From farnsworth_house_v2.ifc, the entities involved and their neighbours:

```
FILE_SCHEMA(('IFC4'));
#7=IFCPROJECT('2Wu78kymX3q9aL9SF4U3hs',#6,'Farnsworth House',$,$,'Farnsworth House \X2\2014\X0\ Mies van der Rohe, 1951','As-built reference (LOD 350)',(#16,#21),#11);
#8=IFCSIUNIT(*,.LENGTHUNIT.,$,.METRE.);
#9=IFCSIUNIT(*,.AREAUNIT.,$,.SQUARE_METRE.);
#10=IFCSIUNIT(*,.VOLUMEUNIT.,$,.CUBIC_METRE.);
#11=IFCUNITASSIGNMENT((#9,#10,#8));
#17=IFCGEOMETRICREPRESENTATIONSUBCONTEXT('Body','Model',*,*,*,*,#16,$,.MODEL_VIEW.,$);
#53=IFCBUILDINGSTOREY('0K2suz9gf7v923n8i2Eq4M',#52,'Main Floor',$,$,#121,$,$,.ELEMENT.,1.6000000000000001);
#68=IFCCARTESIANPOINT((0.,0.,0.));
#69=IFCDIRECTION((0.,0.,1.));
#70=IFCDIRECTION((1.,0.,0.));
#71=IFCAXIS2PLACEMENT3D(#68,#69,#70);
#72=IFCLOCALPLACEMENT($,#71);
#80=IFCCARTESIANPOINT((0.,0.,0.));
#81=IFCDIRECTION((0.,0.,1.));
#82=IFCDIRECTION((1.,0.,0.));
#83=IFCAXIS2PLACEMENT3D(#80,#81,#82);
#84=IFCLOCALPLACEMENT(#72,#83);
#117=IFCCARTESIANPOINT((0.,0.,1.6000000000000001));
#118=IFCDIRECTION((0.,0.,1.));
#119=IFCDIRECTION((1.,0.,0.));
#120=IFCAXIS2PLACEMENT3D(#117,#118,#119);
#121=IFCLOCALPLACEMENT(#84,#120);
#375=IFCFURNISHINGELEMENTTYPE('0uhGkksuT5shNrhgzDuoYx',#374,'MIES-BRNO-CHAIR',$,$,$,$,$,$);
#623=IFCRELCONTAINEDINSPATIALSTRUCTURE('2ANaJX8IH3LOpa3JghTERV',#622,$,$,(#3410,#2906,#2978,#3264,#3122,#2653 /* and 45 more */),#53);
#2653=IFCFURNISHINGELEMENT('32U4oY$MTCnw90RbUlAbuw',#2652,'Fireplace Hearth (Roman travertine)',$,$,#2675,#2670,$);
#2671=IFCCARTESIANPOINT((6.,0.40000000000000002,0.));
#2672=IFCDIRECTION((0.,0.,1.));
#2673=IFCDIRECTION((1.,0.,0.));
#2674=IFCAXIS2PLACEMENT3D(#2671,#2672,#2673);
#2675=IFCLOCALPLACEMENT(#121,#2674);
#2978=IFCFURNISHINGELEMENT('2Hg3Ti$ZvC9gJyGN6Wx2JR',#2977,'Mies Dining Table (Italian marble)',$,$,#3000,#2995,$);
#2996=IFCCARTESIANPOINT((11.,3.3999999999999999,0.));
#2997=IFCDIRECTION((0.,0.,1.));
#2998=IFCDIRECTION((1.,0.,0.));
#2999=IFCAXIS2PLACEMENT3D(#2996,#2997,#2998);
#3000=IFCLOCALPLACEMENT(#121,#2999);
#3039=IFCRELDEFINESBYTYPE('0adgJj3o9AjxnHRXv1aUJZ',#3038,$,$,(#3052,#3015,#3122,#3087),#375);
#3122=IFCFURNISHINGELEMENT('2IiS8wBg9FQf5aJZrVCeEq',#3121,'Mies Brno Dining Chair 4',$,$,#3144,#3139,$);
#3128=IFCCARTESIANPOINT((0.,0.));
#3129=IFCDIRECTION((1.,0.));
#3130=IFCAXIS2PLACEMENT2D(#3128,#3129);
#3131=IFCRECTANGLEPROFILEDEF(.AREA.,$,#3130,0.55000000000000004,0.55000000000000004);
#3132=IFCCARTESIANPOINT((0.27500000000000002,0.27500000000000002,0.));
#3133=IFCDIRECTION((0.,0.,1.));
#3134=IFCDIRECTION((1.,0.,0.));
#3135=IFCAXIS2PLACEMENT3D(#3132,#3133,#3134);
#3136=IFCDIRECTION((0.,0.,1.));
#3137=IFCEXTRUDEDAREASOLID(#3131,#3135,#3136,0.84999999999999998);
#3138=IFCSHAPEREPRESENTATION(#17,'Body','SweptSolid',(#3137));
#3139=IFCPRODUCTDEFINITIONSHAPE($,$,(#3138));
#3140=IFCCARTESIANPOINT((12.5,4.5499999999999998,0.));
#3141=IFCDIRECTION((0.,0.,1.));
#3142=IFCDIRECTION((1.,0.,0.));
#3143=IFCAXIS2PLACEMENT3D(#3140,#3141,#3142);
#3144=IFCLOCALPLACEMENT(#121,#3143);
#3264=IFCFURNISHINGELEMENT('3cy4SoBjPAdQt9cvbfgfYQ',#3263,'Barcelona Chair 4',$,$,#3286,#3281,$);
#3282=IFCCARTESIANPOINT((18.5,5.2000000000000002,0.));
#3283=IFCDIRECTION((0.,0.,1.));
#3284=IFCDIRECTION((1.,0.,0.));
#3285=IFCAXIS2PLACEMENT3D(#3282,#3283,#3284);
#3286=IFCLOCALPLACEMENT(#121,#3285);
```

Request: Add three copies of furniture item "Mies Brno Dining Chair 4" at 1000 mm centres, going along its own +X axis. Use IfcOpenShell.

```python
import ifcopenshell
import ifcopenshell.api.geometry
import ifcopenshell.api.root
import ifcopenshell.util.element
import ifcopenshell.util.placement
import ifcopenshell.util.unit

model = ifcopenshell.open("farnsworth_house_v2.ifc")
unit_scale = ifcopenshell.util.unit.calculate_unit_scale(model)


def reuse_history(source, copy):
    """copy_class also copies each property set's owner history, people and application; keep the originals."""
    for rel in copy.IsDefinedBy:
        if rel.is_a("IfcRelDefinesByProperties") and (history := rel.RelatingPropertyDefinition.OwnerHistory):
            rel.RelatingPropertyDefinition.OwnerHistory = source.OwnerHistory
            ifcopenshell.util.element.remove_deep2(model, history)


source = model.by_guid("2IiS8wBg9FQf5aJZrVCeEq")
base = ifcopenshell.util.placement.get_local_placement(source.ObjectPlacement)
step = base[:3, 0] * 1 / unit_scale

for i in range(1, 4):
    copy = ifcopenshell.api.root.copy_class(model, product=source)
    copy.Representation = ifcopenshell.util.element.copy_deep(
        model, source.Representation, exclude=["IfcGeometricRepresentationContext", "IfcRepresentationMap"]
    )
    reuse_history(source, copy)
    matrix = base.copy()
    matrix[:3, 3] += i * step
    print("added at", matrix[:3, 3].round(3) + 0.0)
    ifcopenshell.api.geometry.edit_object_placement(model, product=copy, matrix=matrix, is_si=False)

model.write("farnsworth_house_v2-out.ifc")
```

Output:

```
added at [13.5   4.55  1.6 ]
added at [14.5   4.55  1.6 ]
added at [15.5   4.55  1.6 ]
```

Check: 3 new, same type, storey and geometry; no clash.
